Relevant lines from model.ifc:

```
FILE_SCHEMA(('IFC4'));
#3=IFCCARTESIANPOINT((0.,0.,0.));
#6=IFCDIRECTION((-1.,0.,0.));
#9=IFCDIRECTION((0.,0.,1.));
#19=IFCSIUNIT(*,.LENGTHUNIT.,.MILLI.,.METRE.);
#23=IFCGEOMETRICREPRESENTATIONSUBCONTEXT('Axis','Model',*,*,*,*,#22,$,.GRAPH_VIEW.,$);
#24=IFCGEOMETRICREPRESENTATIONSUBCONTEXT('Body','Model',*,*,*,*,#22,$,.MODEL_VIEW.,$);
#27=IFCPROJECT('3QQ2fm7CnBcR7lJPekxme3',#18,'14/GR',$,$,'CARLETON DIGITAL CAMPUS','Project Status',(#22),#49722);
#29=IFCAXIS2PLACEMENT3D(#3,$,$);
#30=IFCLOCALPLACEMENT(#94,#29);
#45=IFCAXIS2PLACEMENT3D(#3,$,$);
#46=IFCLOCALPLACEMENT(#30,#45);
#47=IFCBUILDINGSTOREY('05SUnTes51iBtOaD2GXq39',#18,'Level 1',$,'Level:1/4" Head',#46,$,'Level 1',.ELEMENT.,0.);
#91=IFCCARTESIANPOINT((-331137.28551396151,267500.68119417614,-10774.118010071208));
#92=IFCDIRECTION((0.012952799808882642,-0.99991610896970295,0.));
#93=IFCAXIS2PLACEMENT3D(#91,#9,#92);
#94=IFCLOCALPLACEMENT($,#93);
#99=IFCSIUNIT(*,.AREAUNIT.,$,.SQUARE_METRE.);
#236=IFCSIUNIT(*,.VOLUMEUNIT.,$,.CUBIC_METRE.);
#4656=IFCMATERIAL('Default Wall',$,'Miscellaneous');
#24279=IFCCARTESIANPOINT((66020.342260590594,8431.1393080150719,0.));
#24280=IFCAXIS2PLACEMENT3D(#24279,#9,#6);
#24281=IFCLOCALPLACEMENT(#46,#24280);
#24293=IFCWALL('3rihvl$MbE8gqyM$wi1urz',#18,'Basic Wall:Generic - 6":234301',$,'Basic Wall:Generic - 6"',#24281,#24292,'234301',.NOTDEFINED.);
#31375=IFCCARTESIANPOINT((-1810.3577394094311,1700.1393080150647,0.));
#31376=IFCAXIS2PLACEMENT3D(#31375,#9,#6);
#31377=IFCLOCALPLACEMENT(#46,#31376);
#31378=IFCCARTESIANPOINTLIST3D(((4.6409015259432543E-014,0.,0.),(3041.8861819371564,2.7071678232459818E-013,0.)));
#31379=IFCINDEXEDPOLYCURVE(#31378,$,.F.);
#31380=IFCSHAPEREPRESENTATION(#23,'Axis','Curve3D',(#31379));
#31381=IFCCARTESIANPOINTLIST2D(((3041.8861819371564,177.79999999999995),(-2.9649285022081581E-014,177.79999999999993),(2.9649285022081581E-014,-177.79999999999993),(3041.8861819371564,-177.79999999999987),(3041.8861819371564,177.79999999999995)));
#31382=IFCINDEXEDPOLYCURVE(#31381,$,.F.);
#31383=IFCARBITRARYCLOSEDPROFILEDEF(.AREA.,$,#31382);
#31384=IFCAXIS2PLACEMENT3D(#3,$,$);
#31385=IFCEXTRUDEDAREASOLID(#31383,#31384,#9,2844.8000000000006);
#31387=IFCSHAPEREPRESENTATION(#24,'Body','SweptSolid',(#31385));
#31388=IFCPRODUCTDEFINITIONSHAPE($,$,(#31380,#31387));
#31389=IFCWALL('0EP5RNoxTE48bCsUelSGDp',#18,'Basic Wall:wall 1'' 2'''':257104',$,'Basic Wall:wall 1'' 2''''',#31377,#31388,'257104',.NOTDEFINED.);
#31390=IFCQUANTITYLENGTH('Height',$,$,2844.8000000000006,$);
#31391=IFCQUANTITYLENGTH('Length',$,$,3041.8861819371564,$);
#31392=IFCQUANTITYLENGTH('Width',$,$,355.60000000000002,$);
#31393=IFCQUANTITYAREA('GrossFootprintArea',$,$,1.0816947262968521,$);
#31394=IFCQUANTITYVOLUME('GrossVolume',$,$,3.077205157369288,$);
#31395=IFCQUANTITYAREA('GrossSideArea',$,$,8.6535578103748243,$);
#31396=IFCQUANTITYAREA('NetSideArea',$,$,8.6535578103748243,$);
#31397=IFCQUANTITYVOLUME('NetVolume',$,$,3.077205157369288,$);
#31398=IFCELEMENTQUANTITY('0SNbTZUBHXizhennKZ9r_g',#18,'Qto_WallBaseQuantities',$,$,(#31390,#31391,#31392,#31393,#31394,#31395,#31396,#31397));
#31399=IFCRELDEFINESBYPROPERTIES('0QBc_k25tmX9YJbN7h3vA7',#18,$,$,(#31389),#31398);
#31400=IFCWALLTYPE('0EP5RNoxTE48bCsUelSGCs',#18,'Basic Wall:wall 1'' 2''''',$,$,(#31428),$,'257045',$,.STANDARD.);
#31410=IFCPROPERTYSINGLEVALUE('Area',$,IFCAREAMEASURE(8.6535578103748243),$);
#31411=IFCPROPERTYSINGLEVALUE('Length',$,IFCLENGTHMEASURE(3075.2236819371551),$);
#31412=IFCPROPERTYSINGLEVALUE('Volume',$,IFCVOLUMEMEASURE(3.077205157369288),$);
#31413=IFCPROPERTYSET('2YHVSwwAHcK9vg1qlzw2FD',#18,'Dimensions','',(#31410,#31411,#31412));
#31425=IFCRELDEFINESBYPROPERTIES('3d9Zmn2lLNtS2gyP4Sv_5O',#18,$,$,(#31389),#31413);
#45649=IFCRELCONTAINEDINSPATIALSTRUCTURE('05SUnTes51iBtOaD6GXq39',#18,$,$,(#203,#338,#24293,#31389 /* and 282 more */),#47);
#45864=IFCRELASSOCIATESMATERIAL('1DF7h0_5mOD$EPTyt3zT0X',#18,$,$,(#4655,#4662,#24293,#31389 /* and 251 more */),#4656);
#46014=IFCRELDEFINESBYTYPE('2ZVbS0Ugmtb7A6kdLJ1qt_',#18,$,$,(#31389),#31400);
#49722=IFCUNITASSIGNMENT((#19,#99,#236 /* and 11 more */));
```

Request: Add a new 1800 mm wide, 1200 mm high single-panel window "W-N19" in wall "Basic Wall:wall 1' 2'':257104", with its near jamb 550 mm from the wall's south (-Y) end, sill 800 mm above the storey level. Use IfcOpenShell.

```python
import numpy as np
import ifcopenshell
import ifcopenshell.api.feature
import ifcopenshell.api.geometry
import ifcopenshell.api.pset
import ifcopenshell.api.root
import ifcopenshell.api.spatial
import ifcopenshell.geom
import ifcopenshell.util.element
import ifcopenshell.util.placement
import ifcopenshell.util.representation
import ifcopenshell.util.shape
import ifcopenshell.util.unit

model = ifcopenshell.open("model.ifc")
unit_scale = ifcopenshell.util.unit.calculate_unit_scale(model)
area_scale = ifcopenshell.util.unit.calculate_unit_scale(model, "AREAUNIT")
volume_scale = ifcopenshell.util.unit.calculate_unit_scale(model, "VOLUMEUNIT")
settings = ifcopenshell.geom.settings()


def volume(element):
    """Net volume in cubic metres, openings subtracted."""
    shape = ifcopenshell.geom.create_shape(settings, element)
    return ifcopenshell.util.shape.get_volume(shape.geometry)


wall = model.by_guid("0EP5RNoxTE48bCsUelSGDp")
storey = ifcopenshell.util.element.get_container(wall, ifc_class="IfcBuildingStorey")
context = ifcopenshell.util.representation.get_context(model, "Model", "Body", "MODEL_VIEW")
before = volume(wall)

width, height, from_end, sill = 1.8, 1.2, 0.55, 0.8  # metres

# The wall runs along its own X axis, and the end named is its -X end.
wall_shape = ifcopenshell.geom.create_shape(settings, wall)
x, y, z = ifcopenshell.util.shape.get_vertices(wall_shape.geometry).T
start = x.min() + from_end
face, thickness = float(y.min()), float(y.max() - y.min())
wall_matrix = ifcopenshell.util.placement.get_local_placement(wall.ObjectPlacement)
level = ifcopenshell.util.placement.get_local_placement(storey.ObjectPlacement)[2, 3]


def in_wall(x, y):
    """Placement at x, y metres in the wall's axes, at sill height."""
    matrix = wall_matrix.copy()
    matrix[:, 3] = wall_matrix @ np.array([x / unit_scale, y / unit_scale, 0.0, 1.0])
    matrix[2, 3] = level + sill / unit_scale
    return matrix


# Opening: a box that overshoots both wall faces by 50 mm.
opening = ifcopenshell.api.root.create_entity(model, ifc_class="IfcOpeningElement", predefined_type="OPENING")
box = ifcopenshell.api.geometry.add_wall_representation(
    model, context=context, length=width, height=height, thickness=thickness + 0.1
)
ifcopenshell.api.geometry.assign_representation(model, product=opening, representation=box)
ifcopenshell.api.geometry.edit_object_placement(model, product=opening, matrix=in_wall(start, face - 0.05), is_si=False)
ifcopenshell.api.feature.add_feature(model, feature=opening, element=wall)

window = ifcopenshell.api.root.create_entity(model, ifc_class="IfcWindow", name="W-N19", predefined_type="WINDOW")
window.OverallWidth, window.OverallHeight = width / unit_scale, height / unit_scale
window.PartitioningType = "SINGLE_PANEL"
body = ifcopenshell.api.geometry.add_window_representation(
    model,
    context=context,
    overall_width=window.OverallWidth,
    overall_height=window.OverallHeight,
    partition_type="SINGLE_PANEL",
)
ifcopenshell.api.geometry.assign_representation(model, product=window, representation=body)
ifcopenshell.api.spatial.assign_container(model, products=[window], relating_structure=storey)
ifcopenshell.api.feature.add_filling(model, opening=opening, element=window)

# Centre the window in the wall's thickness.
ifcopenshell.api.geometry.edit_object_placement(model, product=window, matrix=in_wall(start, face), is_si=False)
window_shape = ifcopenshell.geom.create_shape(settings, window)
depth = ifcopenshell.util.shape.get_vertices(window_shape.geometry)[:, 1]
offset = face + thickness / 2 - (depth.min() + depth.max()) / 2
ifcopenshell.api.geometry.edit_object_placement(model, product=window, matrix=in_wall(start, offset), is_si=False)

after = volume(wall)

# Update the wall's stored quantities.
qto = model.by_id(ifcopenshell.util.element.get_pset(wall, "Qto_WallBaseQuantities", should_inherit=False)["id"])
ifcopenshell.api.pset.edit_qto(model, qto=qto, properties={
    "NetSideArea": after / thickness / area_scale,
    "NetVolume": after / volume_scale,
})
pset = model.by_id(ifcopenshell.util.element.get_pset(wall, "Dimensions", should_inherit=False)["id"])
ifcopenshell.api.pset.edit_pset(model, pset=pset, properties={
    "Area": model.create_entity("IfcAreaMeasure", after / thickness / area_scale),
    "Volume": model.create_entity("IfcVolumeMeasure", after / volume_scale),
})

print(f"wall volume {before:.3f} -> {after:.3f} m3")

model.write("model-out.ifc")
```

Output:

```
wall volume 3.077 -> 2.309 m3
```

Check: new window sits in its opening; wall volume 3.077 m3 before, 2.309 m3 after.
